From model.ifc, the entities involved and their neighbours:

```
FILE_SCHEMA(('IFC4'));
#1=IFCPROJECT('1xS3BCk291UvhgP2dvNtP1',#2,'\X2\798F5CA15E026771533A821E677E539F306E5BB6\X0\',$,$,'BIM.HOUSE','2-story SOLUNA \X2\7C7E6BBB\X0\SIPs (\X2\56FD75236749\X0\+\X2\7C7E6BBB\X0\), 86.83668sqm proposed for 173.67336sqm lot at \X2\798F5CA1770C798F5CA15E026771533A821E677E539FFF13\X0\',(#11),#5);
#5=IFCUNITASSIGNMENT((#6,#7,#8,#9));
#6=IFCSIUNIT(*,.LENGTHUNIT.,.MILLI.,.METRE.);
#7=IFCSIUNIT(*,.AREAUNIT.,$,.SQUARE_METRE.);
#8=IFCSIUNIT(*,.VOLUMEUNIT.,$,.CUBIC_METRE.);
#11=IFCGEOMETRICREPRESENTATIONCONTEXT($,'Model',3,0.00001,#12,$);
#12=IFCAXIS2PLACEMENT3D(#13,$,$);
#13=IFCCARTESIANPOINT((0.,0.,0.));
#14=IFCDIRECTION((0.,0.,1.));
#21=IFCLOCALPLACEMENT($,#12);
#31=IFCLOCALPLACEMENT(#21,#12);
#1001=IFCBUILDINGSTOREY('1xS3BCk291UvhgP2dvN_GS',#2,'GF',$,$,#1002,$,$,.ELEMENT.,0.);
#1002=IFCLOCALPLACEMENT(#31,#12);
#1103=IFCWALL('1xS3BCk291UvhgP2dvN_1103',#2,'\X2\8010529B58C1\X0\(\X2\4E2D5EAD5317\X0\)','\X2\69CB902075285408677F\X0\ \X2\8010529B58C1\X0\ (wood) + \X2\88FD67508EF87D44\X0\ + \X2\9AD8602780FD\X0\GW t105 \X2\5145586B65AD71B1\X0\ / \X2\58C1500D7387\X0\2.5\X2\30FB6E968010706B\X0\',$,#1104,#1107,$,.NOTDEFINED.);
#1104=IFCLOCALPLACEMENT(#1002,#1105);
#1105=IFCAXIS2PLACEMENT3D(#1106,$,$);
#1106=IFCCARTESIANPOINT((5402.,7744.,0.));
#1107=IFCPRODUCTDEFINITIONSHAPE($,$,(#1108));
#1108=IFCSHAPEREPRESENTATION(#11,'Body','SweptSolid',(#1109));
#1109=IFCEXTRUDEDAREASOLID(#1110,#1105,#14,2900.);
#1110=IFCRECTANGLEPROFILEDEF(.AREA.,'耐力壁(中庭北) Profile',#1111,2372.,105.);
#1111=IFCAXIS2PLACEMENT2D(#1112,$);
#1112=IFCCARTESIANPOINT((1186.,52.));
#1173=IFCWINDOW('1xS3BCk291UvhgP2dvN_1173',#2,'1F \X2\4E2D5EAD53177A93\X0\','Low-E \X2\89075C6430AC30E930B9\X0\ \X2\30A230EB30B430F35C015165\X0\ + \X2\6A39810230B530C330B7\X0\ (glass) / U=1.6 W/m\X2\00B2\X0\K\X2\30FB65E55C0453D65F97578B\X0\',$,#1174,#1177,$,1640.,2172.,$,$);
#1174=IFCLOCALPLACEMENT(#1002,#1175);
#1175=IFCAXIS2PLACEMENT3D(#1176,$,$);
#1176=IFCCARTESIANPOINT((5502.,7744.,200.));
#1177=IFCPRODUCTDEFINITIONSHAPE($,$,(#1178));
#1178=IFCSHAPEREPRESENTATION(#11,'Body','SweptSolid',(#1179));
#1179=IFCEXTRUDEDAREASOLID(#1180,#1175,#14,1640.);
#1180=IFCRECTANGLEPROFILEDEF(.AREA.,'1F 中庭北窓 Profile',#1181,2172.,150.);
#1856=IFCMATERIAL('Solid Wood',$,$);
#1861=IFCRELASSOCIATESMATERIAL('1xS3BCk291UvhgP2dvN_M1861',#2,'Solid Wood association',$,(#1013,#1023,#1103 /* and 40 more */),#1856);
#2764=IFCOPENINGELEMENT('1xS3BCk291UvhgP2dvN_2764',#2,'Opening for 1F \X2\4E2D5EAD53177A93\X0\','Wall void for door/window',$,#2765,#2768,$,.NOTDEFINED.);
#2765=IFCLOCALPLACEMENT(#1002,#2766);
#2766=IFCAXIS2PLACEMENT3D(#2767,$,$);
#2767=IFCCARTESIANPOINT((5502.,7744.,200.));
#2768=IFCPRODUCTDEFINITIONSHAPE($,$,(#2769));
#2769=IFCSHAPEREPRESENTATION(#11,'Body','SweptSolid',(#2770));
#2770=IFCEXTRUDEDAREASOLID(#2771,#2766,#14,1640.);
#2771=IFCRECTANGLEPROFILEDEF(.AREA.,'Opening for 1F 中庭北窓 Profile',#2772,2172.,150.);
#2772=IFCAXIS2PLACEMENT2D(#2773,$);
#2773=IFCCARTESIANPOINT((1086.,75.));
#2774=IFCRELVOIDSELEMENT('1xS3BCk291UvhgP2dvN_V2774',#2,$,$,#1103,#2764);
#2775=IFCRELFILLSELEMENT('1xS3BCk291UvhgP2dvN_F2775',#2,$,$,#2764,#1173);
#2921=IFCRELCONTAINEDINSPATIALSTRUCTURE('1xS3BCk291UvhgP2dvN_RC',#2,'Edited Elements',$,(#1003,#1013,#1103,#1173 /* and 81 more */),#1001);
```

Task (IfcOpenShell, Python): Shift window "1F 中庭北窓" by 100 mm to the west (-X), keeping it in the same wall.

```python
import ifcopenshell
import ifcopenshell.api.geometry
import ifcopenshell.util.placement
import ifcopenshell.util.unit

model = ifcopenshell.open("model.ifc")
unit_scale = ifcopenshell.util.unit.calculate_unit_scale(model)

window = model.by_guid("1xS3BCk291UvhgP2dvN_1173")
opening = window.FillsVoids[0].RelatingOpeningElement
wall = opening.VoidsElements[0].RelatingBuildingElement

wall_matrix = ifcopenshell.util.placement.get_local_placement(wall.ObjectPlacement)
shift = wall_matrix[:3, 0] * -0.1 / unit_scale
before = ifcopenshell.util.placement.get_local_placement(window.ObjectPlacement)[:3, 3].copy()

# The window is not placed relative to its opening, so move both.
for product in (opening, window):
    matrix = ifcopenshell.util.placement.get_local_placement(product.ObjectPlacement)
    matrix[:3, 3] += shift
    ifcopenshell.api.geometry.edit_object_placement(model, product=product, matrix=matrix, is_si=False)

after = ifcopenshell.util.placement.get_local_placement(window.ObjectPlacement)[:3, 3]
print("window moved by", (after - before).round(3) + 0.0)

model.write("model_rev.ifc")
```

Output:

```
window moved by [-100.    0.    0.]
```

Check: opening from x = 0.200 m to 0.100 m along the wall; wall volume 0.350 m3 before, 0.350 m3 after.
